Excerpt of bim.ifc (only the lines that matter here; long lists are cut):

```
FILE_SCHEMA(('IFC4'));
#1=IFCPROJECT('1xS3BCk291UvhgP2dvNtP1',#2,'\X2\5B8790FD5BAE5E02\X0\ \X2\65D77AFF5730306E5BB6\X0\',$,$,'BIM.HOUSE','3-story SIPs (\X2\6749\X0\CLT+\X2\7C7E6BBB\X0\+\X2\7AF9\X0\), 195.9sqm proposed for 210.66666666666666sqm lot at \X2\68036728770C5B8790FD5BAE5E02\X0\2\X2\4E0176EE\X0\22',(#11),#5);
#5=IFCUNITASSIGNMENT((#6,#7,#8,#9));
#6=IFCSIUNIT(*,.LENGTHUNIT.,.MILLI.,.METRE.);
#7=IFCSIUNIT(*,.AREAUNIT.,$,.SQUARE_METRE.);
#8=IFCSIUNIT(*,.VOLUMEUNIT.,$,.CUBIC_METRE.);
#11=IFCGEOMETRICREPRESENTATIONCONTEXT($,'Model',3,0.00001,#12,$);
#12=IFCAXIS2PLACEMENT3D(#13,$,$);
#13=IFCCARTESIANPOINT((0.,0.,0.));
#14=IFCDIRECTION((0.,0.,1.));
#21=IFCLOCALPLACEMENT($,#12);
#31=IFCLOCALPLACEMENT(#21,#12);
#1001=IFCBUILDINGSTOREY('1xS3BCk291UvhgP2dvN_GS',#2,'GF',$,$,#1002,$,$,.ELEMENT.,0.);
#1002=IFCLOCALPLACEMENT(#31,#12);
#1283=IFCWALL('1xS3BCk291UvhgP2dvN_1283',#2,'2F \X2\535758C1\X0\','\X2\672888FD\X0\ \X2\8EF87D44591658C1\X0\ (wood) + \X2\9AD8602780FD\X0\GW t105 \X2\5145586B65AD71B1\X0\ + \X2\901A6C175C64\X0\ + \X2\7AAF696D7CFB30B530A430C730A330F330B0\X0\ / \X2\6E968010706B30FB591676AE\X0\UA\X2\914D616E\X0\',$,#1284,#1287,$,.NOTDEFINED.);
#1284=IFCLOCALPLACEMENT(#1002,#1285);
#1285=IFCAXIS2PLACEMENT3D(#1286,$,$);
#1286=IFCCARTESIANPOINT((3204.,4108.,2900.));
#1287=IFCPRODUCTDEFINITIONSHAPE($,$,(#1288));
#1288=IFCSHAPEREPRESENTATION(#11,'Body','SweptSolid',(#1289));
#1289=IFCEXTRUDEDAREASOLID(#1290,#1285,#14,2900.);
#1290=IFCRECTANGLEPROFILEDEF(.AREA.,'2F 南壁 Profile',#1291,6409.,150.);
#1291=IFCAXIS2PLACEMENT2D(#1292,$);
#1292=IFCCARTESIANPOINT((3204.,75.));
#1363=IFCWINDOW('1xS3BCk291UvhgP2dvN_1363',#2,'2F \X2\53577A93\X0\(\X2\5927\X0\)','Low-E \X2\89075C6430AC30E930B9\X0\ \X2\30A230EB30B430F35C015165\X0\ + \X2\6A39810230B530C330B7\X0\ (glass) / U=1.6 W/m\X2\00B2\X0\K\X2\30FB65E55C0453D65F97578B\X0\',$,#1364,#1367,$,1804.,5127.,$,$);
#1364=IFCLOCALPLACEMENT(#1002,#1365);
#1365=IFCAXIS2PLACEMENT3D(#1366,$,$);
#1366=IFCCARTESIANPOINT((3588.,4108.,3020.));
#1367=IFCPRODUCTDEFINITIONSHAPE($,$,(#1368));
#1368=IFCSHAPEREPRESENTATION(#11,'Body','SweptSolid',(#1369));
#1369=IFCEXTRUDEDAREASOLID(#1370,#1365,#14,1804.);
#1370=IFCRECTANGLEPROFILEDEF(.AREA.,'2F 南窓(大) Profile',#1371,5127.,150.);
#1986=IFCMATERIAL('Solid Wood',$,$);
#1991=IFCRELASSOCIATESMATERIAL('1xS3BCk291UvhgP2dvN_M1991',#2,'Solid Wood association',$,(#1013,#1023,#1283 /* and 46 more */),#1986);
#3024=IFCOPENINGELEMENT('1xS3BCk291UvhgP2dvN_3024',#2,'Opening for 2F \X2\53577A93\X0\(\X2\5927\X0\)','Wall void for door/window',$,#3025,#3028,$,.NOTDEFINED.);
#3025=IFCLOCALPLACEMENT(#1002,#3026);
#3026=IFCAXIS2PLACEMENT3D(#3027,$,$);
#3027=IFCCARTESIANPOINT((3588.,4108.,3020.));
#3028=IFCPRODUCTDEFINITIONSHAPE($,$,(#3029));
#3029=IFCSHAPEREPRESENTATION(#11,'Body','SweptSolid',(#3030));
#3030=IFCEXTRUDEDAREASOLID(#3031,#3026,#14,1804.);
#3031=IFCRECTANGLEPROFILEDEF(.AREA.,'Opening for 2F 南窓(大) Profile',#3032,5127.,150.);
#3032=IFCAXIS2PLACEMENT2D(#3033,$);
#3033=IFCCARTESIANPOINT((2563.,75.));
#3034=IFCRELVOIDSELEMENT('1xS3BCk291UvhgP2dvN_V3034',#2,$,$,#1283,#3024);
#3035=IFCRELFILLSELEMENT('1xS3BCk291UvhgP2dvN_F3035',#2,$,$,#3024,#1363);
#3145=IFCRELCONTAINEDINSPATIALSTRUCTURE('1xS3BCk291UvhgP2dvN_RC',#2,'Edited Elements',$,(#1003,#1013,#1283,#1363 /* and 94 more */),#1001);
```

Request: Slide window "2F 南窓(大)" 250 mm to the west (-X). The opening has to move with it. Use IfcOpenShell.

```python
import ifcopenshell
import ifcopenshell.api.geometry
import ifcopenshell.util.placement
import ifcopenshell.util.unit

model = ifcopenshell.open("bim.ifc")
unit_scale = ifcopenshell.util.unit.calculate_unit_scale(model)

window = model.by_guid("1xS3BCk291UvhgP2dvN_1363")
opening = window.FillsVoids[0].RelatingOpeningElement
wall = opening.VoidsElements[0].RelatingBuildingElement

wall_matrix = ifcopenshell.util.placement.get_local_placement(wall.ObjectPlacement)
shift = wall_matrix[:3, 0] * -0.25 / unit_scale
before = ifcopenshell.util.placement.get_local_placement(window.ObjectPlacement)[:3, 3].copy()

# The window is not placed relative to its opening, so move both.
for product in (opening, window):
    matrix = ifcopenshell.util.placement.get_local_placement(product.ObjectPlacement)
    matrix[:3, 3] += shift
    ifcopenshell.api.geometry.edit_object_placement(model, product=product, matrix=matrix, is_si=False)

after = ifcopenshell.util.placement.get_local_placement(window.ObjectPlacement)[:3, 3]
print("window moved by", (after - before).round(3) + 0.0)

model.write("bim-out.ifc")
```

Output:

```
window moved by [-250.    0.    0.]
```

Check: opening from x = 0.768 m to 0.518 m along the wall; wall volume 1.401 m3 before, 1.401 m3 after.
